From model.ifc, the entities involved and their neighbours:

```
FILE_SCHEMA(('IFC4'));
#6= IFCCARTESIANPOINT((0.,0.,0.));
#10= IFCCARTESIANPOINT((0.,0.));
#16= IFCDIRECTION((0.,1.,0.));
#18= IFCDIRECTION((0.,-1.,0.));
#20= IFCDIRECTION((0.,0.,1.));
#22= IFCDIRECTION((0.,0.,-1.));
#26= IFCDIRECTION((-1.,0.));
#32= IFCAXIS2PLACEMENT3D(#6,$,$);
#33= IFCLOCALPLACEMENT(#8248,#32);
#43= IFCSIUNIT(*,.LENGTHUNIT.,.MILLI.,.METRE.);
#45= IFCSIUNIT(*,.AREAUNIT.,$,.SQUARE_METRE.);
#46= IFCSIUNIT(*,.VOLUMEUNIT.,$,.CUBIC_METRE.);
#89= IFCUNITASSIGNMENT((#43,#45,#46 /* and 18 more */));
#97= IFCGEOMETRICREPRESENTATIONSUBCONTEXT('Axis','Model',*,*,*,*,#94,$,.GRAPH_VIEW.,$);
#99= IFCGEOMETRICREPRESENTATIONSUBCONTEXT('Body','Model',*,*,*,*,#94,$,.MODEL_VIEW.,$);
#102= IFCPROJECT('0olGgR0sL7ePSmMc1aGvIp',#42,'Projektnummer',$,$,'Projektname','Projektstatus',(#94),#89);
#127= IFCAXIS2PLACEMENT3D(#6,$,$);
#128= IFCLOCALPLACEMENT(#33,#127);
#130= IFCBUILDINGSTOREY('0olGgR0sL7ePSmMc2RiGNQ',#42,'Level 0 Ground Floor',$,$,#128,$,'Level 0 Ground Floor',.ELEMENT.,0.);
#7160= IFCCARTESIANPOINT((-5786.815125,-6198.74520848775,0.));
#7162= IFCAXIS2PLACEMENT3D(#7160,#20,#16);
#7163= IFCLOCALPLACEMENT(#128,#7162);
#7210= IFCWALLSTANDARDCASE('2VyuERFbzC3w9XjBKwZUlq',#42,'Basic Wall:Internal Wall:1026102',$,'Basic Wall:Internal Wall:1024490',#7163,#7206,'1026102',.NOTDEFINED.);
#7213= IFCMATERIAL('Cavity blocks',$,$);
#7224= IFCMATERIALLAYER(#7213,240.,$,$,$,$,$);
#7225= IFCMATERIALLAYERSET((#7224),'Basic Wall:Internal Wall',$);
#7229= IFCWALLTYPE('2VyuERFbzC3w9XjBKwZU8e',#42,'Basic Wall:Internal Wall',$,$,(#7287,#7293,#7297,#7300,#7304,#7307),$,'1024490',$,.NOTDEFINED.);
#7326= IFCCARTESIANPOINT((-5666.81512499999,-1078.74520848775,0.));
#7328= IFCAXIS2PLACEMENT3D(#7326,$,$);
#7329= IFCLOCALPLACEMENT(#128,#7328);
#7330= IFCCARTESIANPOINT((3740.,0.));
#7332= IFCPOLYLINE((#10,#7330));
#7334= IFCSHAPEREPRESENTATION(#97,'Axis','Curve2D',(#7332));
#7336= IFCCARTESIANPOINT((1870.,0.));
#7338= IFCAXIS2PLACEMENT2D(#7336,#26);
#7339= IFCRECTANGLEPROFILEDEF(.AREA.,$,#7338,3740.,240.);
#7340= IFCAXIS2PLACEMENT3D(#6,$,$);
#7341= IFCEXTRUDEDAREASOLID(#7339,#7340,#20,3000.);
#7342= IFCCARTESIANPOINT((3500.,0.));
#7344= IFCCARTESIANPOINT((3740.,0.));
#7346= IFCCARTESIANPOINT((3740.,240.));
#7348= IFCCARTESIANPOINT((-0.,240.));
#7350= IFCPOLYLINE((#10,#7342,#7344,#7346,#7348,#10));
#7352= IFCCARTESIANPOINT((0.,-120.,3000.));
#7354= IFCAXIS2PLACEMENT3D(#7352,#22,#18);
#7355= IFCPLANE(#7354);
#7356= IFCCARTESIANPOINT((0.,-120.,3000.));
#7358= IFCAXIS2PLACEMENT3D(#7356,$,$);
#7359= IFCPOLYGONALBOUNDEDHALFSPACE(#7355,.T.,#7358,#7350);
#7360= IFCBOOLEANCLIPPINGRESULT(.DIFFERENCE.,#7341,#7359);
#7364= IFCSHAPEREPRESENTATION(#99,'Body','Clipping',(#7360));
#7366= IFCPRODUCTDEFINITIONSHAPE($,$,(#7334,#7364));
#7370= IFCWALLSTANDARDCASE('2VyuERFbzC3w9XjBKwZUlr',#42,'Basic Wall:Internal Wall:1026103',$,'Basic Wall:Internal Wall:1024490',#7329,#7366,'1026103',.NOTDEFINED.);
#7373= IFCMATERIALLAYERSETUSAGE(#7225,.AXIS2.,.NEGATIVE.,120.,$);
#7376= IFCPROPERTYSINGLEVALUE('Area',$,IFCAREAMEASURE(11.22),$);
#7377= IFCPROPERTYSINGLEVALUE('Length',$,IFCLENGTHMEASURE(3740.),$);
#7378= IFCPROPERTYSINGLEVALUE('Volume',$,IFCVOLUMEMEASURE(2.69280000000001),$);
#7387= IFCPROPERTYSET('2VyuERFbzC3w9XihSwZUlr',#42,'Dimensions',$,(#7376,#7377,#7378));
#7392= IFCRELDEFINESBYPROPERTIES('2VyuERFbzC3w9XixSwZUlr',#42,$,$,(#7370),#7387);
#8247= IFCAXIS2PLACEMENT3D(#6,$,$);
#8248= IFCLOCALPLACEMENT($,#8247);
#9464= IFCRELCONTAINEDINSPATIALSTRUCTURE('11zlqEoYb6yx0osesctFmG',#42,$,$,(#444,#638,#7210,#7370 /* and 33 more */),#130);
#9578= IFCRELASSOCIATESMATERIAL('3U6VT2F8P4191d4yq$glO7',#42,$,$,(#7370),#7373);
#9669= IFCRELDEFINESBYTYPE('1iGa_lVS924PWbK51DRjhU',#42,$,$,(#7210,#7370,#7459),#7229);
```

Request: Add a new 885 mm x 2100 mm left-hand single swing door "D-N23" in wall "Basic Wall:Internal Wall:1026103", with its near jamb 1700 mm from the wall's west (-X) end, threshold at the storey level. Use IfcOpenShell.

```python
import numpy as np
import ifcopenshell
import ifcopenshell.api.feature
import ifcopenshell.api.geometry
import ifcopenshell.api.pset
import ifcopenshell.api.root
import ifcopenshell.api.spatial
import ifcopenshell.geom
import ifcopenshell.util.element
import ifcopenshell.util.placement
import ifcopenshell.util.representation
import ifcopenshell.util.shape
import ifcopenshell.util.unit

model = ifcopenshell.open("model.ifc")
unit_scale = ifcopenshell.util.unit.calculate_unit_scale(model)
area_scale = ifcopenshell.util.unit.calculate_unit_scale(model, "AREAUNIT")
volume_scale = ifcopenshell.util.unit.calculate_unit_scale(model, "VOLUMEUNIT")
settings = ifcopenshell.geom.settings()


def volume(element):
    """Net volume in cubic metres, openings subtracted."""
    shape = ifcopenshell.geom.create_shape(settings, element)
    return ifcopenshell.util.shape.get_volume(shape.geometry)


wall = model.by_id(7370)
storey = ifcopenshell.util.element.get_container(wall, ifc_class="IfcBuildingStorey")
context = ifcopenshell.util.representation.get_context(model, "Model", "Body", "MODEL_VIEW")
before = volume(wall)

width, height, from_end, sill = 0.885, 2.1, 1.7, 0.0  # metres

# The wall runs along its own X axis, and the end named is its -X end.
wall_shape = ifcopenshell.geom.create_shape(settings, wall)
x, y, z = ifcopenshell.util.shape.get_vertices(wall_shape.geometry).T
start = x.min() + from_end
face, thickness = float(y.min()), float(y.max() - y.min())
wall_matrix = ifcopenshell.util.placement.get_local_placement(wall.ObjectPlacement)
level = ifcopenshell.util.placement.get_local_placement(storey.ObjectPlacement)[2, 3]


def in_wall(x, y):
    """Placement at x, y metres in the wall's axes, at sill height."""
    matrix = wall_matrix.copy()
    matrix[:, 3] = wall_matrix @ np.array([x / unit_scale, y / unit_scale, 0.0, 1.0])
    matrix[2, 3] = level + sill / unit_scale
    return matrix


# Opening: a box that overshoots both wall faces by 50 mm.
opening = ifcopenshell.api.root.create_entity(model, ifc_class="IfcOpeningElement", predefined_type="OPENING")
box = ifcopenshell.api.geometry.add_wall_representation(
    model, context=context, length=width, height=height, thickness=thickness + 0.1
)
ifcopenshell.api.geometry.assign_representation(model, product=opening, representation=box)
ifcopenshell.api.geometry.edit_object_placement(model, product=opening, matrix=in_wall(start, face - 0.05), is_si=False)
ifcopenshell.api.feature.add_feature(model, feature=opening, element=wall)

door = ifcopenshell.api.root.create_entity(model, ifc_class="IfcDoor", name="D-N23", predefined_type="DOOR")
door.OverallWidth, door.OverallHeight = width / unit_scale, height / unit_scale
door.OperationType = "SINGLE_SWING_LEFT"
body = ifcopenshell.api.geometry.add_door_representation(
    model,
    context=context,
    overall_width=door.OverallWidth,
    overall_height=door.OverallHeight,
    operation_type="SINGLE_SWING_LEFT",
    lining_properties={"LiningDepth": thickness / unit_scale, "ThresholdDepth": thickness / unit_scale},
)
ifcopenshell.api.geometry.assign_representation(model, product=door, representation=body)
ifcopenshell.api.spatial.assign_container(model, products=[door], relating_structure=storey)
ifcopenshell.api.feature.add_filling(model, opening=opening, element=door)

# The lining spans the wall, so the door starts at the wall face.
ifcopenshell.api.geometry.edit_object_placement(model, product=door, matrix=in_wall(start, face), is_si=False)

after = volume(wall)

# Update the wall's stored quantities.
pset = model.by_id(ifcopenshell.util.element.get_pset(wall, "Dimensions", should_inherit=False)["id"])
ifcopenshell.api.pset.edit_pset(model, pset=pset, properties={
    "Area": model.create_entity("IfcAreaMeasure", after / thickness / area_scale),
    "Volume": model.create_entity("IfcVolumeMeasure", after / volume_scale),
})

print(f"wall volume {before:.3f} -> {after:.3f} m3")

model.write("model_v2.ifc")
```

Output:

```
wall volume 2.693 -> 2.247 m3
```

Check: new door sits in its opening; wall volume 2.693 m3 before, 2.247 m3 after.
